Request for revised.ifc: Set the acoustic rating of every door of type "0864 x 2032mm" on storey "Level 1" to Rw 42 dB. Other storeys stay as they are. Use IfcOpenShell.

First a look at what the model holds.

```python
import ifcopenshell
import ifcopenshell.util.element

model = ifcopenshell.open("revised.ifc")
print(model.schema)
storey = next(s for s in model.by_type("IfcBuildingStorey") if s.Name == "Level 1")
doors = [e for e in ifcopenshell.util.element.get_decomposition(storey) if e.is_a("IfcDoor")]
seen = {}
for e in doors:
    element_type = ifcopenshell.util.element.get_type(e)
    key = (element_type.Name if element_type != e and element_type else None, ifcopenshell.util.element.get_pset(e, "Pset_DoorCommon", "AcousticRating"))
    seen[key] = seen.get(key, 0) + 1
for (name, value), count in sorted(seen.items(), key=str):
    print(count, "x", name, "|", value)
```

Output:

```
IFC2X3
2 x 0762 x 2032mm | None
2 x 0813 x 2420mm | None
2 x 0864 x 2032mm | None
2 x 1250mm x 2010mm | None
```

```python
import ifcopenshell
import ifcopenshell.api.pset
import ifcopenshell.util.element

model = ifcopenshell.open("revised.ifc")

storey = next(s for s in model.by_type("IfcBuildingStorey") if s.Name == "Level 1")
doors = [e for e in ifcopenshell.util.element.get_decomposition(storey) if e.is_a("IfcDoor")]

count = 0
for e in doors:
    element_type = ifcopenshell.util.element.get_type(e)
    if element_type in (None, e) or element_type.Name != "0864 x 2032mm":
        continue
    # add_pset returns the element's existing set when there is one.
    pset = ifcopenshell.api.pset.add_pset(model, product=e, name="Pset_DoorCommon")
    ifcopenshell.api.pset.edit_pset(model, pset=pset, properties={"AcousticRating": "Rw 42 dB"})
    count += 1

print(count, "doors updated")

model.write("revised_rev.ifc")
```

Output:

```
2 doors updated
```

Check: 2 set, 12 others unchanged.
